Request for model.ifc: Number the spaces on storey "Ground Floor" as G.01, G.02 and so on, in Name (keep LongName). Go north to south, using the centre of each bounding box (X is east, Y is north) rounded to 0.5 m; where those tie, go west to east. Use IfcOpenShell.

First a look at what the model holds.

```python
import ifcopenshell
import ifcopenshell.util.element
import ifcopenshell.util.placement

model = ifcopenshell.open("model.ifc")
print(model.schema)
storey = next(s for s in model.by_type("IfcBuildingStorey") if s.Name == "Ground Floor")
spaces = [e for e in ifcopenshell.util.element.get_decomposition(storey) if e.is_a("IfcSpace")]
for e in sorted(spaces, key=lambda e: e.id()):
    origin = ifcopenshell.util.placement.get_local_placement(e.ObjectPlacement)[:3, 3]
    print(e.id(), e.Name, e.LongName, origin.round(2) + 0.0, sep=" | ")
```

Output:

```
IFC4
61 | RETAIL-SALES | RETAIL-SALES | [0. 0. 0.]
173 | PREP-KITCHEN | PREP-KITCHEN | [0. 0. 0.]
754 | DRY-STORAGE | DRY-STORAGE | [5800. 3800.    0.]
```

```python
import ifcopenshell
import ifcopenshell.geom
import ifcopenshell.util.element
import ifcopenshell.util.shape

model = ifcopenshell.open("model.ifc")
settings = ifcopenshell.geom.settings()
settings.set("use-world-coords", True)


def centre(element):
    shape = ifcopenshell.geom.create_shape(settings, element)
    return ifcopenshell.util.shape.get_bbox_centroid(shape.geometry)


storey = next(s for s in model.by_type("IfcBuildingStorey") if s.Name == "Ground Floor")
spaces = [e for e in ifcopenshell.util.element.get_decomposition(storey) if e.is_a("IfcSpace")]

# Insertion points can sit at a corner or the storey origin, so sort by the geometry (in metres).
centres = {e: centre(e) for e in spaces}
spaces.sort(key=lambda e: (-round(centres[e][1] / 0.5), centres[e][0]))

for i, e in enumerate(spaces, start=1):
    number = f"G.{i:02d}"
    e.Name = number
    print(e.id(), number)

model.write("model_rev.ifc")
```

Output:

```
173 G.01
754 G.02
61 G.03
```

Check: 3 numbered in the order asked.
